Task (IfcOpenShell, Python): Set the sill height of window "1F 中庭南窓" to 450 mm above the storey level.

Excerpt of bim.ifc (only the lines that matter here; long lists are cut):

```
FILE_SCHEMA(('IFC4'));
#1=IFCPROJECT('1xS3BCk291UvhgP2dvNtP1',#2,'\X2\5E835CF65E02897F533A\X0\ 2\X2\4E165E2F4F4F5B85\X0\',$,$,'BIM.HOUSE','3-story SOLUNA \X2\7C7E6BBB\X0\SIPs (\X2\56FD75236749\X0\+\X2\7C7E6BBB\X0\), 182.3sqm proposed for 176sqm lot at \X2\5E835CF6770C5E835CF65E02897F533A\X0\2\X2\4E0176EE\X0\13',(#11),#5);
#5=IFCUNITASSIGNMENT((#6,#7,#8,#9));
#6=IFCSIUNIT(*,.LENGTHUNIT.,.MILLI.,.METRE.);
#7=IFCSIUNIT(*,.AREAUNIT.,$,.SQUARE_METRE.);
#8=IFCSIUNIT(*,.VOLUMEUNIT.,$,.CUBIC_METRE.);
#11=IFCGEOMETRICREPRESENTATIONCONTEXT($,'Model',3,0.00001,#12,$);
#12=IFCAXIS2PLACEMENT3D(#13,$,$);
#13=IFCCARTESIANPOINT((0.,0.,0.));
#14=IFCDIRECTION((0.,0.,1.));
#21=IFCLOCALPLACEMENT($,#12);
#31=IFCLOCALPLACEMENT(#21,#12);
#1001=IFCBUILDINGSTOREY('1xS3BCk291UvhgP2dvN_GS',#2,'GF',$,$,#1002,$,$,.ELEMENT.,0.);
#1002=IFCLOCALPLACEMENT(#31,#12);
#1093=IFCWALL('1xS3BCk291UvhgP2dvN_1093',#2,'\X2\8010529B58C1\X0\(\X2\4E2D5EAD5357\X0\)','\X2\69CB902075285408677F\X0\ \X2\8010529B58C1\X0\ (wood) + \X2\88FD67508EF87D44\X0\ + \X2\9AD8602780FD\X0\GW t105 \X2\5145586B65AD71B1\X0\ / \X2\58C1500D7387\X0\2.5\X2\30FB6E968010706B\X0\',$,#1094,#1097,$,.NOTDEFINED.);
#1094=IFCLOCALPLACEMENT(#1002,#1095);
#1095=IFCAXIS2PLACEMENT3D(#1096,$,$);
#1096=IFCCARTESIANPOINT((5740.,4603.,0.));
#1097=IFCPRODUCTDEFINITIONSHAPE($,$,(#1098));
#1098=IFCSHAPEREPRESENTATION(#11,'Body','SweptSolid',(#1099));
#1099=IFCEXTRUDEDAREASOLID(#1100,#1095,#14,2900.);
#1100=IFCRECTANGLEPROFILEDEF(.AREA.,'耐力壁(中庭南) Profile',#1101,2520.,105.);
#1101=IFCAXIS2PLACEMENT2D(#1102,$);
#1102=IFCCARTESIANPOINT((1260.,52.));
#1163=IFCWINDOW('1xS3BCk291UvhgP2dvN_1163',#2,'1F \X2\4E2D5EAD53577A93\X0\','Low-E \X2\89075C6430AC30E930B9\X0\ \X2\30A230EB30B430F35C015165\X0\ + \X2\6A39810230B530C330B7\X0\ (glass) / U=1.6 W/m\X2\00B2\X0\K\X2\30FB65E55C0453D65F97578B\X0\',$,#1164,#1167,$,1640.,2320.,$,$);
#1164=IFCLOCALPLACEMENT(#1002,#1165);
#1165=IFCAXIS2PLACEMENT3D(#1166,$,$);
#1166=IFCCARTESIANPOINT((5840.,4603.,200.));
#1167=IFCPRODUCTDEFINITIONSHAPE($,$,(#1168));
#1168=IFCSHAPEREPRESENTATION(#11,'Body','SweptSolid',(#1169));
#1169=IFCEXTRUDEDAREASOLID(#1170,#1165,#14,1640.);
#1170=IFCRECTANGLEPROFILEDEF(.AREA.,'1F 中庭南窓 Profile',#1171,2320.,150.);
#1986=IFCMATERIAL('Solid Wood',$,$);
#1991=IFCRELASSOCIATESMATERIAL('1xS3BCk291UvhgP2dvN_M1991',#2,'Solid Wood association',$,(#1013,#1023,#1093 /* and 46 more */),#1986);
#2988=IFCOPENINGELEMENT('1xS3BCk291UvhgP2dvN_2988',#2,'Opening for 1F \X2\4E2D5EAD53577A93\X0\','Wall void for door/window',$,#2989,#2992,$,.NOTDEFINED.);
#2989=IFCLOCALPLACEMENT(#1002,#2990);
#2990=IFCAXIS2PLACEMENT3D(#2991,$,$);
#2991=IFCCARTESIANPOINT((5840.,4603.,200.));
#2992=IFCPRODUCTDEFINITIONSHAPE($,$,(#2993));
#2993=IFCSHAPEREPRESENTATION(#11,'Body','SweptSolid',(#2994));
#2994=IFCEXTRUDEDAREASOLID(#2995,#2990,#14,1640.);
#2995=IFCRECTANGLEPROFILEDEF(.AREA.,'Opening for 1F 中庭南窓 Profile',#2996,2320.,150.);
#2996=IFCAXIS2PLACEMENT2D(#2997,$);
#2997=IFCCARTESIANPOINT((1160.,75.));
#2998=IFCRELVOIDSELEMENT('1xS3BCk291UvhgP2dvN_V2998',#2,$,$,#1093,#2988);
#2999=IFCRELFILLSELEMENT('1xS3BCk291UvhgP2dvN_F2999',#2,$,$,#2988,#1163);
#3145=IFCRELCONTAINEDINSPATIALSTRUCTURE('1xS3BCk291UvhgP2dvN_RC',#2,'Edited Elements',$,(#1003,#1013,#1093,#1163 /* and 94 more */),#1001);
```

```python
import numpy as np
import ifcopenshell
import ifcopenshell.api.geometry
import ifcopenshell.geom
import ifcopenshell.util.element
import ifcopenshell.util.placement
import ifcopenshell.util.shape
import ifcopenshell.util.unit

model = ifcopenshell.open("bim.ifc")
unit_scale = ifcopenshell.util.unit.calculate_unit_scale(model)

window = model.by_guid("1xS3BCk291UvhgP2dvN_1163")
opening = window.FillsVoids[0].RelatingOpeningElement
storey = ifcopenshell.util.element.get_container(window, ifc_class="IfcBuildingStorey")
level = ifcopenshell.util.placement.get_local_placement(storey.ObjectPlacement)[2, 3]

# The opening's origin need not be at the sill, so measure its lowest point.
shape = ifcopenshell.geom.create_shape(ifcopenshell.geom.settings(), opening)
bottom = ifcopenshell.util.shape.get_shape_bottom_elevation(shape, shape.geometry) / unit_scale
dz = level + 0.45 / unit_scale - bottom

shift = np.array([0.0, 0.0, dz])
# The window is not placed relative to its opening, so move both.
for product in (opening, window):
    matrix = ifcopenshell.util.placement.get_local_placement(product.ObjectPlacement)
    matrix[:3, 3] += shift
    ifcopenshell.api.geometry.edit_object_placement(model, product=product, matrix=matrix, is_si=False)

print(f"moved by {dz * unit_scale:+.3f} m")

model.write("bim-out.ifc")
```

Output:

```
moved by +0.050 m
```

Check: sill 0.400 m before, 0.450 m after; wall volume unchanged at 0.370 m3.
